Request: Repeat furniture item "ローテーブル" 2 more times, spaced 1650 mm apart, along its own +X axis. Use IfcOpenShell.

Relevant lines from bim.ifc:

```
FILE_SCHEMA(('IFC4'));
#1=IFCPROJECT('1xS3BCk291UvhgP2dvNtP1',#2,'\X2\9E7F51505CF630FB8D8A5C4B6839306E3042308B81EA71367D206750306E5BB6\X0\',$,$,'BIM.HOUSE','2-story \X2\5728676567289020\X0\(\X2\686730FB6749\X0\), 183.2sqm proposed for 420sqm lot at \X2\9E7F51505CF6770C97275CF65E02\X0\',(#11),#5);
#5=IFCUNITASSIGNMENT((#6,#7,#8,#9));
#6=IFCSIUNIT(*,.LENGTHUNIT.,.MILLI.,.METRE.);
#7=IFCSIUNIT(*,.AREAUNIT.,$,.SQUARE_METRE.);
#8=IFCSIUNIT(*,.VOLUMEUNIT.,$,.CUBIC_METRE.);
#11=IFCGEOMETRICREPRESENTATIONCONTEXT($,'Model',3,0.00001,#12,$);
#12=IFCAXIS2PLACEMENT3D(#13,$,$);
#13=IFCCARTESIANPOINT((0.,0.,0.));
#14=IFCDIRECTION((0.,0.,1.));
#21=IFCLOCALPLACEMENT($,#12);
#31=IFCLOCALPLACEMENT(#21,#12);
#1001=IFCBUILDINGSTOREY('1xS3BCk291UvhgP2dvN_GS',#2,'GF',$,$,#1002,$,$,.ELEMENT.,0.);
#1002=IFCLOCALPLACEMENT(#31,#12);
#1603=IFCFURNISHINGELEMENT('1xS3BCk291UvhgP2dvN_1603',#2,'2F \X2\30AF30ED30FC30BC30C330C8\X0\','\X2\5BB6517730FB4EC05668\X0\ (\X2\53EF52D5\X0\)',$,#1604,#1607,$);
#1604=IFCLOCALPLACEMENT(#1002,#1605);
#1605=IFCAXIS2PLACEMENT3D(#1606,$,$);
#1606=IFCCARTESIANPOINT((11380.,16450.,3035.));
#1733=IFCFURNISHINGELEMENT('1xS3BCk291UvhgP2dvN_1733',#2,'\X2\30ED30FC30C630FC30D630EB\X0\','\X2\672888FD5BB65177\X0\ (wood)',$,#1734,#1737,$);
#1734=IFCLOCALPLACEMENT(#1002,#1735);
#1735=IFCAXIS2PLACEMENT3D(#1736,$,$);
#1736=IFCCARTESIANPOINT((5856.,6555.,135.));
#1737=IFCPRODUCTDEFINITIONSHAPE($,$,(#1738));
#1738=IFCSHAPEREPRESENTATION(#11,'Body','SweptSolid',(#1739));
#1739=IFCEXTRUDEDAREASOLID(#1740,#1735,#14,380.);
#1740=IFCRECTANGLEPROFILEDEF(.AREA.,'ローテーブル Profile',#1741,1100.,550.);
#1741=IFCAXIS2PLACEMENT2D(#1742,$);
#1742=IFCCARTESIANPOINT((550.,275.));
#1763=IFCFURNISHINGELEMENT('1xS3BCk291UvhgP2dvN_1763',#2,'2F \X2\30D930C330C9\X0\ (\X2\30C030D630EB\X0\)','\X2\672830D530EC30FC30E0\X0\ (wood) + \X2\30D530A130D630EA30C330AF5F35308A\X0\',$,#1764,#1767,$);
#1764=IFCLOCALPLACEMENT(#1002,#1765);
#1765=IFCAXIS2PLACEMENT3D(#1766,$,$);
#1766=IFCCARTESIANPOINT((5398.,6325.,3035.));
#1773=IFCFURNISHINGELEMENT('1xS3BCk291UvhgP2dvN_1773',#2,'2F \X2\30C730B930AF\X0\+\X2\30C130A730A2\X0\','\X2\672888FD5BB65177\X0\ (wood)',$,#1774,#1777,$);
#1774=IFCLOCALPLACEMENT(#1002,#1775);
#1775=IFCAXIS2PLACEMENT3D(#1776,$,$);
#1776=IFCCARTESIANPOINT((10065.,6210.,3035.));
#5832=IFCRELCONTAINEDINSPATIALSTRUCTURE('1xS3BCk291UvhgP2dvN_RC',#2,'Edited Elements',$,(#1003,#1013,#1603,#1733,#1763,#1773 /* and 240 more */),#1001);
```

```python
import ifcopenshell
import ifcopenshell.api.geometry
import ifcopenshell.api.root
import ifcopenshell.util.element
import ifcopenshell.util.placement

model = ifcopenshell.open("bim.ifc")


def reuse_history(source, copy):
    """copy_class also copies each property set's owner history, people and application; keep the originals."""
    for rel in copy.IsDefinedBy:
        if rel.is_a("IfcRelDefinesByProperties") and (history := rel.RelatingPropertyDefinition.OwnerHistory):
            rel.RelatingPropertyDefinition.OwnerHistory = source.OwnerHistory
            ifcopenshell.util.element.remove_deep2(model, history)


source = model.by_guid("1xS3BCk291UvhgP2dvN_1733")
base = ifcopenshell.util.placement.get_local_placement(source.ObjectPlacement)
step = base[:3, 0] * 1650.0

for i in range(1, 3):
    copy = ifcopenshell.api.root.copy_class(model, product=source)
    copy.Representation = ifcopenshell.util.element.copy_deep(
        model, source.Representation, exclude=["IfcGeometricRepresentationContext", "IfcRepresentationMap"]
    )
    reuse_history(source, copy)
    matrix = base.copy()
    matrix[:3, 3] += i * step
    print("added at", matrix[:3, 3].round(3) + 0.0)
    ifcopenshell.api.geometry.edit_object_placement(model, product=copy, matrix=matrix, is_si=False)

model.write("bim-out.ifc")
```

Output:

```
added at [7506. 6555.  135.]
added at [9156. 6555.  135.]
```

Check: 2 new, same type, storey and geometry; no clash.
